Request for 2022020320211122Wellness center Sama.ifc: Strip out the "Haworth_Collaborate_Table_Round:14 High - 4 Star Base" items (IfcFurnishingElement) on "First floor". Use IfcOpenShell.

First a look at what the model holds.

```python
import ifcopenshell
import ifcopenshell.util.element

model = ifcopenshell.open("2022020320211122Wellness center Sama.ifc")
print(model.schema)
storey = next(s for s in model.by_type("IfcBuildingStorey") if s.Name == "First floor")
furniture = [e for e in ifcopenshell.util.element.get_decomposition(storey) if e.is_a("IfcFurnishingElement")]
seen = {}
for e in furniture:
    element_type = ifcopenshell.util.element.get_type(e)
    name = element_type.Name if element_type not in (None, e) else None
    seen[name] = seen.get(name, 0) + 1
for name, count in sorted(seen.items(), key=str):
    print(count, "x", name)
```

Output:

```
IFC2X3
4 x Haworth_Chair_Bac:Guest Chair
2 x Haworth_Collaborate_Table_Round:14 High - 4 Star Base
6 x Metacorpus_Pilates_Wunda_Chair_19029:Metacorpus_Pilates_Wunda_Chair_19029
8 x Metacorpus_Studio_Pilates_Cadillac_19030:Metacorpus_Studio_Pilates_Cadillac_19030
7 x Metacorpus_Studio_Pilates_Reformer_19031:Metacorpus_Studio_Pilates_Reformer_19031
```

```python
import ifcopenshell
import ifcopenshell.api.root
import ifcopenshell.util.element

model = ifcopenshell.open("2022020320211122Wellness center Sama.ifc")

storey = next(s for s in model.by_type("IfcBuildingStorey") if s.Name == "First floor")
furniture = [e for e in ifcopenshell.util.element.get_decomposition(storey) if e.is_a("IfcFurnishingElement")]
targets = [e for e in furniture if (t := ifcopenshell.util.element.get_type(e)) not in (None, e) and t.Name == "Haworth_Collaborate_Table_Round:14 High - 4 Star Base"]

for e in targets:
    ifcopenshell.api.root.remove_product(model, product=e)
print(len(targets), "removed")

model.write("2022020320211122Wellness center Sama_updated.ifc")
```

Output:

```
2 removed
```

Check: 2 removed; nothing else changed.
